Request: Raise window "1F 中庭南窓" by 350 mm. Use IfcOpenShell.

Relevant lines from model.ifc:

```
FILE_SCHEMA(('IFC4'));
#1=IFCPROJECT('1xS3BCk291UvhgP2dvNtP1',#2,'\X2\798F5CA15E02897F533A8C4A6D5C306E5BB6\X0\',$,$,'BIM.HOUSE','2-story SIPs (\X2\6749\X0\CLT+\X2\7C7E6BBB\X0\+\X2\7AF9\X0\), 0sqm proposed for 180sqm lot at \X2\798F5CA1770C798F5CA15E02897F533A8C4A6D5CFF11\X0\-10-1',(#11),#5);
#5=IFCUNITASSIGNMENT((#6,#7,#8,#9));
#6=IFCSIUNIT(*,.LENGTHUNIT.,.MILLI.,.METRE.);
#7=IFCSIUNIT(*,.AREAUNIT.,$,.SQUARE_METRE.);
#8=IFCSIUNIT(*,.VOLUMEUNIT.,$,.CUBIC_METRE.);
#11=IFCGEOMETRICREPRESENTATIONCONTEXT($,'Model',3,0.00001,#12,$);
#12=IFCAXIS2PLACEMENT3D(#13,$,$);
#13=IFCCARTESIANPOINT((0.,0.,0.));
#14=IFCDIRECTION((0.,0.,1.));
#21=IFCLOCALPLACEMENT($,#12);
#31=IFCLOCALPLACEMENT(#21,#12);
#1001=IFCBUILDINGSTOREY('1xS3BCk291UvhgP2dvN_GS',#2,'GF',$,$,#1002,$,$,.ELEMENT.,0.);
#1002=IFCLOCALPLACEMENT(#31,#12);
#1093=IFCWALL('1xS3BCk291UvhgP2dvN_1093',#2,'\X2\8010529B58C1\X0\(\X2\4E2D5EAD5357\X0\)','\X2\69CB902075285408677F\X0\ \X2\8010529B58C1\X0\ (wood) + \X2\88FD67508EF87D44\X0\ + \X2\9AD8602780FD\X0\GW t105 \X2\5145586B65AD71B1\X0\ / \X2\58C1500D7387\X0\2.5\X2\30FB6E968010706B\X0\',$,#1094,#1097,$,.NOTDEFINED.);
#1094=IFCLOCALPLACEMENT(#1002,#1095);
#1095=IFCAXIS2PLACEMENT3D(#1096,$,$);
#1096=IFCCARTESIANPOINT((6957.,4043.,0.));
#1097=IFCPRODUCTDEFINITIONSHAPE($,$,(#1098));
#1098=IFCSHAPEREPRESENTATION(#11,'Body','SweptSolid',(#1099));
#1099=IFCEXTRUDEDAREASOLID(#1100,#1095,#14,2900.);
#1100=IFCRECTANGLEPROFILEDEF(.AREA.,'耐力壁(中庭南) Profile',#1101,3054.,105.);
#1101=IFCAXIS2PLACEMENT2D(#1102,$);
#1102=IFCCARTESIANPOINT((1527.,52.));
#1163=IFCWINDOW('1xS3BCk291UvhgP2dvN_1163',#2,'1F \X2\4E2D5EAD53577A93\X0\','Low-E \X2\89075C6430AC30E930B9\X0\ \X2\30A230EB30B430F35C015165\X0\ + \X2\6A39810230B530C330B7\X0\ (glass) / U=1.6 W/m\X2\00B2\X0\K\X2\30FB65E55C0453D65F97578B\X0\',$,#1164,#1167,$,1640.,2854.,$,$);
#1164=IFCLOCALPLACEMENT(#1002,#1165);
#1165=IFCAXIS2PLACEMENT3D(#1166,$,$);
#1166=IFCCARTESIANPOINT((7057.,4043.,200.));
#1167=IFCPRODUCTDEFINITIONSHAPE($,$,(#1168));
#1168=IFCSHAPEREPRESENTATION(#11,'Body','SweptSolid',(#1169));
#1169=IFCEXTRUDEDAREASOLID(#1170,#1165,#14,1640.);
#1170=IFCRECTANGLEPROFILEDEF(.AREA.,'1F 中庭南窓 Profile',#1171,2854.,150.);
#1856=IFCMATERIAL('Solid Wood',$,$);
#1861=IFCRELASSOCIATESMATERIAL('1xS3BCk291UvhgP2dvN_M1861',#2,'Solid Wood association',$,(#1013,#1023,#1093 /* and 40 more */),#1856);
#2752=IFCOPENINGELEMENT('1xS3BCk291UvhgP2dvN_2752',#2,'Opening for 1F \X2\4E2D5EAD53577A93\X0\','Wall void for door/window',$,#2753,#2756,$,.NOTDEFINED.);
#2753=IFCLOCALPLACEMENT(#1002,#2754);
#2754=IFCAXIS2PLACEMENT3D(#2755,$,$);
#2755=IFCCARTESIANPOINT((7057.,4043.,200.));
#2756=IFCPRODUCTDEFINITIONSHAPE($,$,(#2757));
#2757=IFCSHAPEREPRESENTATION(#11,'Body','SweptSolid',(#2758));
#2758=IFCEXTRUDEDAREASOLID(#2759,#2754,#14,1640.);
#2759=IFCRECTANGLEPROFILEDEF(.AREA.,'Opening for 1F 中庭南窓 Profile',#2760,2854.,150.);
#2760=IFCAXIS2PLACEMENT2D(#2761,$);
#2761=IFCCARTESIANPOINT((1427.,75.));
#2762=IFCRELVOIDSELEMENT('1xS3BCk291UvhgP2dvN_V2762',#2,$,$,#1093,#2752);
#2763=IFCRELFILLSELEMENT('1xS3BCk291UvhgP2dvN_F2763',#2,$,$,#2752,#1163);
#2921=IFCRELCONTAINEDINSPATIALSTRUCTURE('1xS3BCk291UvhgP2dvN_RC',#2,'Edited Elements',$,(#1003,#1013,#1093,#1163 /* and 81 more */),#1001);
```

```python
import numpy as np
import ifcopenshell
import ifcopenshell.api.geometry
import ifcopenshell.util.placement
import ifcopenshell.util.unit

model = ifcopenshell.open("model.ifc")
unit_scale = ifcopenshell.util.unit.calculate_unit_scale(model)

window = model.by_guid("1xS3BCk291UvhgP2dvN_1163")
opening = window.FillsVoids[0].RelatingOpeningElement
dz = 350.0

shift = np.array([0.0, 0.0, dz])
# The window is not placed relative to its opening, so move both.
for product in (opening, window):
    matrix = ifcopenshell.util.placement.get_local_placement(product.ObjectPlacement)
    matrix[:3, 3] += shift
    ifcopenshell.api.geometry.edit_object_placement(model, product=product, matrix=matrix, is_si=False)

print(f"moved by {dz * unit_scale:+.3f} m")

model.write("model_updated.ifc")
```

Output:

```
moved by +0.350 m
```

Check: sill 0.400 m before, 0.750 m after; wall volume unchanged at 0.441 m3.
